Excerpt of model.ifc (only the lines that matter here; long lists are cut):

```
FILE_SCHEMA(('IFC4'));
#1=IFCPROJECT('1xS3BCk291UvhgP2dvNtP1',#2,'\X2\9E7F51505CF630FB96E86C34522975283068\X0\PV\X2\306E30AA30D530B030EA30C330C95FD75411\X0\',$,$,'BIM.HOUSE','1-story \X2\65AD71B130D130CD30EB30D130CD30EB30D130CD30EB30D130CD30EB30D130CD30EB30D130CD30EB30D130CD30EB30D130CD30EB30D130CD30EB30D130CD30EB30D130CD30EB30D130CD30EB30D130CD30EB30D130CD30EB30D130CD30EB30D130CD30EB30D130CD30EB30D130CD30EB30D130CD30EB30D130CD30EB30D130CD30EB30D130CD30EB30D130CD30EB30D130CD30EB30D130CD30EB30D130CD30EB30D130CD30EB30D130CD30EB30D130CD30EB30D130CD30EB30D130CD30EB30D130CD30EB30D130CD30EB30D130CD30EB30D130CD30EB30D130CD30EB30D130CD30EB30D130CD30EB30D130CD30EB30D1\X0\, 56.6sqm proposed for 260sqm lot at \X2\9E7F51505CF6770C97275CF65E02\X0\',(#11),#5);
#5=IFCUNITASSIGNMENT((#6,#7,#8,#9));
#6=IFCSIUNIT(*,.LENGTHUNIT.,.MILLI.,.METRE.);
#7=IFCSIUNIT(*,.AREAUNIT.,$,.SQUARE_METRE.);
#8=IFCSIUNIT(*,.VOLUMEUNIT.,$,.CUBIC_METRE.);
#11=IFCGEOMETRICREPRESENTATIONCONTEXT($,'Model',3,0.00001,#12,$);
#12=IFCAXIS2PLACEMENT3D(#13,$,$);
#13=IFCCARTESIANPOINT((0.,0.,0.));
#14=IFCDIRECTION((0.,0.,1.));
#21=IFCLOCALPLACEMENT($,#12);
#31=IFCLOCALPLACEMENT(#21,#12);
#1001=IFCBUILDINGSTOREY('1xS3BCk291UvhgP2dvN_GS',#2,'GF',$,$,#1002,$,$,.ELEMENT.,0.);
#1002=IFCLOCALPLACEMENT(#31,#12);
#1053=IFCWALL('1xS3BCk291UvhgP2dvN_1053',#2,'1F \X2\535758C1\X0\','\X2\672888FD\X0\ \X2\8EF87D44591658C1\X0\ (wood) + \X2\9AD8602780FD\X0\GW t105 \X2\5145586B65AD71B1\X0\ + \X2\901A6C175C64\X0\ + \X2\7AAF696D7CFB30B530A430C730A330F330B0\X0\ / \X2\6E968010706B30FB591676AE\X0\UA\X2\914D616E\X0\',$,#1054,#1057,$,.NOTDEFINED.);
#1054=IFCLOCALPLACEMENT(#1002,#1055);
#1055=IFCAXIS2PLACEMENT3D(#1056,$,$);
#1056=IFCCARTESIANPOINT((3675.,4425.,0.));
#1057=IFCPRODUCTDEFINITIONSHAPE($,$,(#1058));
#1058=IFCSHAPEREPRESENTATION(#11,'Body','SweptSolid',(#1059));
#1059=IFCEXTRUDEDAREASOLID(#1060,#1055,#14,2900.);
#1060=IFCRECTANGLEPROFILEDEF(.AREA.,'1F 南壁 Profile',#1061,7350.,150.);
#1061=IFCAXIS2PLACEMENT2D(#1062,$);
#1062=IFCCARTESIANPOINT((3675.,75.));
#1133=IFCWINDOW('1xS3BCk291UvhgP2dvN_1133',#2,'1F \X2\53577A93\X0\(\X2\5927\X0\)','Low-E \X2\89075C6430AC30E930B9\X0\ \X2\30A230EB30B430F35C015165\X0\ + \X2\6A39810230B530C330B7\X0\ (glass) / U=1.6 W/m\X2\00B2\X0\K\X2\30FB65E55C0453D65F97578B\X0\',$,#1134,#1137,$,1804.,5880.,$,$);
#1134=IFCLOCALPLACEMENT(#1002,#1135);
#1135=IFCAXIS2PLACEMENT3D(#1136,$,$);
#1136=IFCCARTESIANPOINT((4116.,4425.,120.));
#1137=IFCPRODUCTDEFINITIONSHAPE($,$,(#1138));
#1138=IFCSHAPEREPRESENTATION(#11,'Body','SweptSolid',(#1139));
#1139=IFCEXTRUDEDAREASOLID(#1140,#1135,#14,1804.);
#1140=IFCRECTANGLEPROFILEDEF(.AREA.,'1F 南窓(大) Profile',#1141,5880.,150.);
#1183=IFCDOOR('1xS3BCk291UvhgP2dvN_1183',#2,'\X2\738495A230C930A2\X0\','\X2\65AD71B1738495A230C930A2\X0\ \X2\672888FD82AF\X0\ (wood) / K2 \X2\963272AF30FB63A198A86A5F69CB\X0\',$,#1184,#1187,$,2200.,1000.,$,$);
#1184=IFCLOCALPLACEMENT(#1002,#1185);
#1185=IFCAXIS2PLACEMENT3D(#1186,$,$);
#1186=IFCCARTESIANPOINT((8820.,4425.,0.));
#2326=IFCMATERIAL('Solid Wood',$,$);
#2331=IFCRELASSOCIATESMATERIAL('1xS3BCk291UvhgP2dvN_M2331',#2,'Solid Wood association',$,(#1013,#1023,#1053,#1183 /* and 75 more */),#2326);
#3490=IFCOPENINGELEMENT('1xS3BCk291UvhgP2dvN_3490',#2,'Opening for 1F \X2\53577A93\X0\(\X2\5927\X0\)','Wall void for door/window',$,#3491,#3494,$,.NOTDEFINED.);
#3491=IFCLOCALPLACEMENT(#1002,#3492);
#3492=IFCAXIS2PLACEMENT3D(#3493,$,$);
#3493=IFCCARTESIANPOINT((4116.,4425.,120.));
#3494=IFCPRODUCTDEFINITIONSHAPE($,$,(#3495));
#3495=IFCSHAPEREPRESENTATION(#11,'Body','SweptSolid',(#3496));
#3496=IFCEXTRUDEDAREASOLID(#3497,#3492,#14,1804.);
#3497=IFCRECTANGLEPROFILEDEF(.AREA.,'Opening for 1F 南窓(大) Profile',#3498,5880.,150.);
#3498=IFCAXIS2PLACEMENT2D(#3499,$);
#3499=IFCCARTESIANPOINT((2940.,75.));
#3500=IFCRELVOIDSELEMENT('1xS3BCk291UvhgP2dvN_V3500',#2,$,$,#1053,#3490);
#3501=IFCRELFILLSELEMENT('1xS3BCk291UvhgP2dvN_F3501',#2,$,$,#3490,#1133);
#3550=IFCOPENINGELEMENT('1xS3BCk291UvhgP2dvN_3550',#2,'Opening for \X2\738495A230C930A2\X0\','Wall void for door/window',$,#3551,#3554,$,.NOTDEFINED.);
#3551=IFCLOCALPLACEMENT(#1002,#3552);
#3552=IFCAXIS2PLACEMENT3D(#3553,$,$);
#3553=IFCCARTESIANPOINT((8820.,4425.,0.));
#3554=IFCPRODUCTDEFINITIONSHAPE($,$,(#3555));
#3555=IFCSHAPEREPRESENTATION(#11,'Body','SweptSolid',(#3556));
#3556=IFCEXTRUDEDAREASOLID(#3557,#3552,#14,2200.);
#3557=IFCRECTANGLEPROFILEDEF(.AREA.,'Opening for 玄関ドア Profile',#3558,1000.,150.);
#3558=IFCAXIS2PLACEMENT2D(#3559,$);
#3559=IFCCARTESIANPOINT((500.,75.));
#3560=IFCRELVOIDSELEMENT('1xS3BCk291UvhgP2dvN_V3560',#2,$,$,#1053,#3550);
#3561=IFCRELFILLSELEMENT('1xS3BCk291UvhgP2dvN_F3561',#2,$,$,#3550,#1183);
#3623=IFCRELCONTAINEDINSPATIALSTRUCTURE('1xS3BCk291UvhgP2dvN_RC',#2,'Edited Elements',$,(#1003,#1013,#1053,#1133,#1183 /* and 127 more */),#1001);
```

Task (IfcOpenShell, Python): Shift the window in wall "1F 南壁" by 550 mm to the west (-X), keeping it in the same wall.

```python
import ifcopenshell
import ifcopenshell.api.geometry
import ifcopenshell.util.placement

model = ifcopenshell.open("model.ifc")

window = model.by_guid("1xS3BCk291UvhgP2dvN_1133")
opening = window.FillsVoids[0].RelatingOpeningElement
wall = opening.VoidsElements[0].RelatingBuildingElement

wall_matrix = ifcopenshell.util.placement.get_local_placement(wall.ObjectPlacement)
shift = wall_matrix[:3, 0] * -550.0
before = ifcopenshell.util.placement.get_local_placement(window.ObjectPlacement)[:3, 3].copy()

# The window is not placed relative to its opening, so move both.
for product in (opening, window):
    matrix = ifcopenshell.util.placement.get_local_placement(product.ObjectPlacement)
    matrix[:3, 3] += shift
    ifcopenshell.api.geometry.edit_object_placement(model, product=product, matrix=matrix, is_si=False)

after = ifcopenshell.util.placement.get_local_placement(window.ObjectPlacement)[:3, 3]
print("window moved by", (after - before).round(3) + 0.0)

model.write("model_v2.ifc")
```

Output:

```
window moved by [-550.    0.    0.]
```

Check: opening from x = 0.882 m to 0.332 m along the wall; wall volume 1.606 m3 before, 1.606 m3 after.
